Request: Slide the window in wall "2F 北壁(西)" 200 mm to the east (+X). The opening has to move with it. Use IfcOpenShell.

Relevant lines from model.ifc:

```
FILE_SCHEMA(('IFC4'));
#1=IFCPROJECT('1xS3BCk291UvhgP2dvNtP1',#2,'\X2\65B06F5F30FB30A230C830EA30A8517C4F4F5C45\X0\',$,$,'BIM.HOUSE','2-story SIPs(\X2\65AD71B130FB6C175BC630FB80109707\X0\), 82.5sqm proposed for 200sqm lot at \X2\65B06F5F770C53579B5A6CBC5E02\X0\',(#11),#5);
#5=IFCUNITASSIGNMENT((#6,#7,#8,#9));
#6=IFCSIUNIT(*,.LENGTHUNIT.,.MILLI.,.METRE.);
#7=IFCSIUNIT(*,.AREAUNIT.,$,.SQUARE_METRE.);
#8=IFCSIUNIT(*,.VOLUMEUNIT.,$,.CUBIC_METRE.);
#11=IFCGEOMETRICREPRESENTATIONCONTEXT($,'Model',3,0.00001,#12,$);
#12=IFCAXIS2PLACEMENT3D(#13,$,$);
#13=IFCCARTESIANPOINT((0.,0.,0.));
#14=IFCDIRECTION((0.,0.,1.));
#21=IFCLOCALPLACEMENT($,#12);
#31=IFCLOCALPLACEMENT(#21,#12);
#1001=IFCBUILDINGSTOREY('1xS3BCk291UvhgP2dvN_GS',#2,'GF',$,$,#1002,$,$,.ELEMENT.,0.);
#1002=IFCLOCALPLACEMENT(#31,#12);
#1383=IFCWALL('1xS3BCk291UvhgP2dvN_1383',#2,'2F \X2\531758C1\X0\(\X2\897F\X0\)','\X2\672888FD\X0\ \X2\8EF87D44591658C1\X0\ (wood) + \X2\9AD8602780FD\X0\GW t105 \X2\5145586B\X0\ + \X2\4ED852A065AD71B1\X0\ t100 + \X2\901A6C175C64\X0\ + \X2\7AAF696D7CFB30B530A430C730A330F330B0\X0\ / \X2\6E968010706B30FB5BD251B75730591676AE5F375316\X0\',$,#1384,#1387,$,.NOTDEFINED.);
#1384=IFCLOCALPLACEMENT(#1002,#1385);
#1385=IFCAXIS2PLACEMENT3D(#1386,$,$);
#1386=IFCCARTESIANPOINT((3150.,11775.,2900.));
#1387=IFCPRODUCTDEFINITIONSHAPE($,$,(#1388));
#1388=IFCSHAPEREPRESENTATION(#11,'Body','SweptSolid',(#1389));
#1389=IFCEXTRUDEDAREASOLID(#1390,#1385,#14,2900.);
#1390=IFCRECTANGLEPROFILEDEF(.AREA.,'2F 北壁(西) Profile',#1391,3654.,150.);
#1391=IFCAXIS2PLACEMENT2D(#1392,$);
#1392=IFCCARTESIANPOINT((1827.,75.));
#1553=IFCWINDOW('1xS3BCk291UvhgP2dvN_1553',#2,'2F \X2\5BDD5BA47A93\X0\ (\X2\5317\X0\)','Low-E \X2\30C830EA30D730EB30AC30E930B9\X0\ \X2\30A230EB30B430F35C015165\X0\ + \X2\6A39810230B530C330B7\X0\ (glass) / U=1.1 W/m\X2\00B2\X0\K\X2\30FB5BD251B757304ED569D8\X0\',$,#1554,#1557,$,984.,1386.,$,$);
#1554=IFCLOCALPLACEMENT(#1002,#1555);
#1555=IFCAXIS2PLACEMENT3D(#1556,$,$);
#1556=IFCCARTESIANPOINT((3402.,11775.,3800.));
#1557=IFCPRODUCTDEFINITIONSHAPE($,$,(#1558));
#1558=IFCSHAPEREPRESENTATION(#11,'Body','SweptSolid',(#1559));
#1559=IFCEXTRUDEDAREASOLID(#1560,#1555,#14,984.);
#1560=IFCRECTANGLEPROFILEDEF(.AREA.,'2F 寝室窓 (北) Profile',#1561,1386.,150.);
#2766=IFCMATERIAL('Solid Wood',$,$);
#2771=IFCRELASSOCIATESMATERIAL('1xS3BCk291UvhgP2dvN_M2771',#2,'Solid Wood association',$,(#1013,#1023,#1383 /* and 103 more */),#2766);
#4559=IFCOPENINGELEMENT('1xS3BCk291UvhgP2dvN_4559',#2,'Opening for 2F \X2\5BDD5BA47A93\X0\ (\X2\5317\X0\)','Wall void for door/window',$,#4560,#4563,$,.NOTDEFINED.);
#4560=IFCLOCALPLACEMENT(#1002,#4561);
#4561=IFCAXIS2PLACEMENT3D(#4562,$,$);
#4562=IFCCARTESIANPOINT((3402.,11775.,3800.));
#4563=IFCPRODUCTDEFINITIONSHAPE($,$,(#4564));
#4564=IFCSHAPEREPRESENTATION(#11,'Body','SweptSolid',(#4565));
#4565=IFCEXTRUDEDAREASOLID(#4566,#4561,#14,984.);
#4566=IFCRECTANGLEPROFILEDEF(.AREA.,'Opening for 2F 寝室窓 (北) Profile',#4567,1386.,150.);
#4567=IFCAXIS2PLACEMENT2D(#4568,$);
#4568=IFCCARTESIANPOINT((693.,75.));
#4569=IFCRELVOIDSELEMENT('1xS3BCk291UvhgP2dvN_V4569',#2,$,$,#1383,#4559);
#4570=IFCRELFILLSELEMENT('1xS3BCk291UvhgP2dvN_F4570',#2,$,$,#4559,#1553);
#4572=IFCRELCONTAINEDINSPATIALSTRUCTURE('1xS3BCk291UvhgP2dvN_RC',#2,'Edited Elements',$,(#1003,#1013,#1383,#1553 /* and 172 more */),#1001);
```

```python
import ifcopenshell
import ifcopenshell.api.geometry
import ifcopenshell.util.placement

model = ifcopenshell.open("model.ifc")

window = model.by_guid("1xS3BCk291UvhgP2dvN_1553")
opening = window.FillsVoids[0].RelatingOpeningElement
wall = opening.VoidsElements[0].RelatingBuildingElement

wall_matrix = ifcopenshell.util.placement.get_local_placement(wall.ObjectPlacement)
shift = wall_matrix[:3, 0] * 200.0
before = ifcopenshell.util.placement.get_local_placement(window.ObjectPlacement)[:3, 3].copy()

# The window is not placed relative to its opening, so move both.
for product in (opening, window):
    matrix = ifcopenshell.util.placement.get_local_placement(product.ObjectPlacement)
    matrix[:3, 3] += shift
    ifcopenshell.api.geometry.edit_object_placement(model, product=product, matrix=matrix, is_si=False)

after = ifcopenshell.util.placement.get_local_placement(window.ObjectPlacement)[:3, 3]
print("window moved by", (after - before).round(3) + 0.0)

model.write("model_rev.ifc")
```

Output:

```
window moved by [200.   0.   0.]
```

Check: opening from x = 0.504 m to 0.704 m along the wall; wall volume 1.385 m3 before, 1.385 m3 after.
